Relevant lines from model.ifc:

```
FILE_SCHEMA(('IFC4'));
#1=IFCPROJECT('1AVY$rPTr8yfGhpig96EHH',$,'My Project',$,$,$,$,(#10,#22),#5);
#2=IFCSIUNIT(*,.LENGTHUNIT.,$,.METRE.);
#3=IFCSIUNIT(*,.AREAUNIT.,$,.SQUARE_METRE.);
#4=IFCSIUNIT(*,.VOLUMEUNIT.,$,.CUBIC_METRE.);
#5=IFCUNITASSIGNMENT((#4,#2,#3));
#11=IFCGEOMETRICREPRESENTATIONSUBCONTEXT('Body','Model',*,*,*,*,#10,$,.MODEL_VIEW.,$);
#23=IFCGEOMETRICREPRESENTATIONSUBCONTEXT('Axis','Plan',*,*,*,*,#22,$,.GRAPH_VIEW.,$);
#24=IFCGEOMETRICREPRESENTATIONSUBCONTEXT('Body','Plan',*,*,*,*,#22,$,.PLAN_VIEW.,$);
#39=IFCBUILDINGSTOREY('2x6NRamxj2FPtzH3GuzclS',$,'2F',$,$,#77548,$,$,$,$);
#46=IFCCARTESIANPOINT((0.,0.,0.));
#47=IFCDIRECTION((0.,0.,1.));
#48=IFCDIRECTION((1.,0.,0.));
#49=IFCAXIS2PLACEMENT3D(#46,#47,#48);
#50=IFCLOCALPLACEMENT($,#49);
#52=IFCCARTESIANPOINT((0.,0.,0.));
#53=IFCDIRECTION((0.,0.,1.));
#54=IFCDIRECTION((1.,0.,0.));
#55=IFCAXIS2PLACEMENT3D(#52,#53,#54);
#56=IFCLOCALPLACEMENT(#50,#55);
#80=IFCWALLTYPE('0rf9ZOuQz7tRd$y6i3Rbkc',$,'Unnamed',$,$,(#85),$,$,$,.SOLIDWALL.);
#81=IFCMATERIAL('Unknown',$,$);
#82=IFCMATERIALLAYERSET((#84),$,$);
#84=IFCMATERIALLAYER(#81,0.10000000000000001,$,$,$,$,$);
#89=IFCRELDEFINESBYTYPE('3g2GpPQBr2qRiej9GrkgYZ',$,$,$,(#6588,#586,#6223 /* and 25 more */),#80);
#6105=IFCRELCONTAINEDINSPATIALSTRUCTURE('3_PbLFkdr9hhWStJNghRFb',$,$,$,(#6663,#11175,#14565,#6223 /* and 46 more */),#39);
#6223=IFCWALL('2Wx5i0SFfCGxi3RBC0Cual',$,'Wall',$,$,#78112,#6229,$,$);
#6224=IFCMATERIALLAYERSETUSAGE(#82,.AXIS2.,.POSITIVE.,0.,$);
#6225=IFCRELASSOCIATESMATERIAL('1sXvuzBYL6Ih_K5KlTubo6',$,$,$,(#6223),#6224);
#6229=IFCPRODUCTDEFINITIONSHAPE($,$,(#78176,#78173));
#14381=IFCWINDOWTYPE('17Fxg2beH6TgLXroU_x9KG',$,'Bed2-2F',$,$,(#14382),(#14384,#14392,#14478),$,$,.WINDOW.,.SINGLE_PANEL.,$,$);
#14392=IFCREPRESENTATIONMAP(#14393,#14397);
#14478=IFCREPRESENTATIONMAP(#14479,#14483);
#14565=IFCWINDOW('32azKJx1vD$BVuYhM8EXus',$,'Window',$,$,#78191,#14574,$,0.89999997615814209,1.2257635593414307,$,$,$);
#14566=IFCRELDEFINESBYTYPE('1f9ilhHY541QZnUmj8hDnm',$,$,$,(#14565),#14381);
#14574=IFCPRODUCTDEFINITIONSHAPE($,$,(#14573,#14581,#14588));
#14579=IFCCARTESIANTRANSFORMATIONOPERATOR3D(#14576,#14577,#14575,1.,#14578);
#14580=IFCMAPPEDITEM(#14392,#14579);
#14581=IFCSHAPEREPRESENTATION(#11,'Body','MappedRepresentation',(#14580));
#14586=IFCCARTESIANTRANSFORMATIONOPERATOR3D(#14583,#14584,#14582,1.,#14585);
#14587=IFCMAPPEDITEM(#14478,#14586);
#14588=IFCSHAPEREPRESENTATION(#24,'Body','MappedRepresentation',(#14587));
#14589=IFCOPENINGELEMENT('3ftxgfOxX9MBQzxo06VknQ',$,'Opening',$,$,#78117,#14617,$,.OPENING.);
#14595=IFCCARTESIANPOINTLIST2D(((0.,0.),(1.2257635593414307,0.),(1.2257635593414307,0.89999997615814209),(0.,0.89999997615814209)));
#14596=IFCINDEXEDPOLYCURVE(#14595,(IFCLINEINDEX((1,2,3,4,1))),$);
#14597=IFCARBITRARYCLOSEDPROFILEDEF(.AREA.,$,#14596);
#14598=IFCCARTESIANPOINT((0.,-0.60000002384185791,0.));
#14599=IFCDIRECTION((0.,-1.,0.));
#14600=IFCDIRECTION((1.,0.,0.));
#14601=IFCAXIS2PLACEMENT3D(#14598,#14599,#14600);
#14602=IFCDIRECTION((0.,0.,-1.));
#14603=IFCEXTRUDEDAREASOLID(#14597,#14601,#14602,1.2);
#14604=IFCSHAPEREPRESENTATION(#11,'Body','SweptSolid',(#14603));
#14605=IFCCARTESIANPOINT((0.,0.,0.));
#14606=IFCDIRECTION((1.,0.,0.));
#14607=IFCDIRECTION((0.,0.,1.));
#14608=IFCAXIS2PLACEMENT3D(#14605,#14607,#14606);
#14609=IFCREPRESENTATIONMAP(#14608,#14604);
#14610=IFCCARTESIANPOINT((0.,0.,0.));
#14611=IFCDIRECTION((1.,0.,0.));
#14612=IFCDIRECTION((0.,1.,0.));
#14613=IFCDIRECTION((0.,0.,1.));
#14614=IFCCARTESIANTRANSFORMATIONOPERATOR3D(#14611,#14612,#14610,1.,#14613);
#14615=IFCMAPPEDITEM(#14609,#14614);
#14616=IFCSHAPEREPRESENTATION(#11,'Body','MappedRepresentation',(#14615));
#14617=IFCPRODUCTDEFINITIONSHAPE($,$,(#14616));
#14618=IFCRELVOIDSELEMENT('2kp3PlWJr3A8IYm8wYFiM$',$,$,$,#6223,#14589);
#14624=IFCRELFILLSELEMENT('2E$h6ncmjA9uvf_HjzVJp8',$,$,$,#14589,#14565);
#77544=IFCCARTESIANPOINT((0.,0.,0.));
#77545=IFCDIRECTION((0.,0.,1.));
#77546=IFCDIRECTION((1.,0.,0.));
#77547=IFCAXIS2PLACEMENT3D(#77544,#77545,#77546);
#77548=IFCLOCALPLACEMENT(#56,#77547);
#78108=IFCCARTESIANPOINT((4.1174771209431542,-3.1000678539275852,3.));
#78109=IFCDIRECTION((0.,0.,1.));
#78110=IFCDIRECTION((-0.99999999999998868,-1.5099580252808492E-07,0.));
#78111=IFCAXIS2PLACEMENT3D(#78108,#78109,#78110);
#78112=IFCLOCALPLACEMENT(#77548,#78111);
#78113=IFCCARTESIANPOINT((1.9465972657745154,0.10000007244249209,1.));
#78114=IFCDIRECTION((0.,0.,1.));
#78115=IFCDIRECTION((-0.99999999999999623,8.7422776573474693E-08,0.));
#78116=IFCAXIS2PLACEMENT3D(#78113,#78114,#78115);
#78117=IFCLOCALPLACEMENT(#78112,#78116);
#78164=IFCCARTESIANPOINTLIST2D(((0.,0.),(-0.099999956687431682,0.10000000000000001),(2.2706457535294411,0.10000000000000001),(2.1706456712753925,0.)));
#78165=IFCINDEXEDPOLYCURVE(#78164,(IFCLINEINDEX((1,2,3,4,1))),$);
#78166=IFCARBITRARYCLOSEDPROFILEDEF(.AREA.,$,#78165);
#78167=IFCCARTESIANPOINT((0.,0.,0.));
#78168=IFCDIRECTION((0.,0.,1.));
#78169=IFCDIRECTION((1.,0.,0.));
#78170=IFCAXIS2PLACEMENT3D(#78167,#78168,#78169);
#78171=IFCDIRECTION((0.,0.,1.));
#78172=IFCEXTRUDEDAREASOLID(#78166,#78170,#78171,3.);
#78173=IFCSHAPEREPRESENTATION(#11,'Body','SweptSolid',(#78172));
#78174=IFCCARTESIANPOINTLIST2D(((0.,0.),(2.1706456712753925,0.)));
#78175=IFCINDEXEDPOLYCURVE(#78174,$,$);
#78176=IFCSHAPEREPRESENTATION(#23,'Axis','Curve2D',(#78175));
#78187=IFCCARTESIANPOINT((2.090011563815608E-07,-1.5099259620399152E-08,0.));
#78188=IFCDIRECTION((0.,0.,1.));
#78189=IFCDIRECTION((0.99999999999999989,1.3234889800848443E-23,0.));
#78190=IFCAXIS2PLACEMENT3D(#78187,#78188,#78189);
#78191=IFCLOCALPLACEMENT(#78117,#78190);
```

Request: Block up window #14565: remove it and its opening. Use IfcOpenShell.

```python
import ifcopenshell
import ifcopenshell.api.feature
import ifcopenshell.api.root
import ifcopenshell.geom
import ifcopenshell.util.shape

model = ifcopenshell.open("model.ifc")
settings = ifcopenshell.geom.settings()


def volume(element):
    """Net volume in cubic metres, openings subtracted."""
    shape = ifcopenshell.geom.create_shape(settings, element)
    return ifcopenshell.util.shape.get_volume(shape.geometry)


window = model.by_guid("32azKJx1vD$BVuYhM8EXus")
opening = window.FillsVoids[0].RelatingOpeningElement
wall = opening.VoidsElements[0].RelatingBuildingElement
before = volume(wall)

ifcopenshell.api.root.remove_product(model, product=window)
ifcopenshell.api.feature.remove_feature(model, feature=opening)

after = volume(wall)

print(f"wall volume {before:.3f} -> {after:.3f} m3")

model.write("model-out.ifc")
```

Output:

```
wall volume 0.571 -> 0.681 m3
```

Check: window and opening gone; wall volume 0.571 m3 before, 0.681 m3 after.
